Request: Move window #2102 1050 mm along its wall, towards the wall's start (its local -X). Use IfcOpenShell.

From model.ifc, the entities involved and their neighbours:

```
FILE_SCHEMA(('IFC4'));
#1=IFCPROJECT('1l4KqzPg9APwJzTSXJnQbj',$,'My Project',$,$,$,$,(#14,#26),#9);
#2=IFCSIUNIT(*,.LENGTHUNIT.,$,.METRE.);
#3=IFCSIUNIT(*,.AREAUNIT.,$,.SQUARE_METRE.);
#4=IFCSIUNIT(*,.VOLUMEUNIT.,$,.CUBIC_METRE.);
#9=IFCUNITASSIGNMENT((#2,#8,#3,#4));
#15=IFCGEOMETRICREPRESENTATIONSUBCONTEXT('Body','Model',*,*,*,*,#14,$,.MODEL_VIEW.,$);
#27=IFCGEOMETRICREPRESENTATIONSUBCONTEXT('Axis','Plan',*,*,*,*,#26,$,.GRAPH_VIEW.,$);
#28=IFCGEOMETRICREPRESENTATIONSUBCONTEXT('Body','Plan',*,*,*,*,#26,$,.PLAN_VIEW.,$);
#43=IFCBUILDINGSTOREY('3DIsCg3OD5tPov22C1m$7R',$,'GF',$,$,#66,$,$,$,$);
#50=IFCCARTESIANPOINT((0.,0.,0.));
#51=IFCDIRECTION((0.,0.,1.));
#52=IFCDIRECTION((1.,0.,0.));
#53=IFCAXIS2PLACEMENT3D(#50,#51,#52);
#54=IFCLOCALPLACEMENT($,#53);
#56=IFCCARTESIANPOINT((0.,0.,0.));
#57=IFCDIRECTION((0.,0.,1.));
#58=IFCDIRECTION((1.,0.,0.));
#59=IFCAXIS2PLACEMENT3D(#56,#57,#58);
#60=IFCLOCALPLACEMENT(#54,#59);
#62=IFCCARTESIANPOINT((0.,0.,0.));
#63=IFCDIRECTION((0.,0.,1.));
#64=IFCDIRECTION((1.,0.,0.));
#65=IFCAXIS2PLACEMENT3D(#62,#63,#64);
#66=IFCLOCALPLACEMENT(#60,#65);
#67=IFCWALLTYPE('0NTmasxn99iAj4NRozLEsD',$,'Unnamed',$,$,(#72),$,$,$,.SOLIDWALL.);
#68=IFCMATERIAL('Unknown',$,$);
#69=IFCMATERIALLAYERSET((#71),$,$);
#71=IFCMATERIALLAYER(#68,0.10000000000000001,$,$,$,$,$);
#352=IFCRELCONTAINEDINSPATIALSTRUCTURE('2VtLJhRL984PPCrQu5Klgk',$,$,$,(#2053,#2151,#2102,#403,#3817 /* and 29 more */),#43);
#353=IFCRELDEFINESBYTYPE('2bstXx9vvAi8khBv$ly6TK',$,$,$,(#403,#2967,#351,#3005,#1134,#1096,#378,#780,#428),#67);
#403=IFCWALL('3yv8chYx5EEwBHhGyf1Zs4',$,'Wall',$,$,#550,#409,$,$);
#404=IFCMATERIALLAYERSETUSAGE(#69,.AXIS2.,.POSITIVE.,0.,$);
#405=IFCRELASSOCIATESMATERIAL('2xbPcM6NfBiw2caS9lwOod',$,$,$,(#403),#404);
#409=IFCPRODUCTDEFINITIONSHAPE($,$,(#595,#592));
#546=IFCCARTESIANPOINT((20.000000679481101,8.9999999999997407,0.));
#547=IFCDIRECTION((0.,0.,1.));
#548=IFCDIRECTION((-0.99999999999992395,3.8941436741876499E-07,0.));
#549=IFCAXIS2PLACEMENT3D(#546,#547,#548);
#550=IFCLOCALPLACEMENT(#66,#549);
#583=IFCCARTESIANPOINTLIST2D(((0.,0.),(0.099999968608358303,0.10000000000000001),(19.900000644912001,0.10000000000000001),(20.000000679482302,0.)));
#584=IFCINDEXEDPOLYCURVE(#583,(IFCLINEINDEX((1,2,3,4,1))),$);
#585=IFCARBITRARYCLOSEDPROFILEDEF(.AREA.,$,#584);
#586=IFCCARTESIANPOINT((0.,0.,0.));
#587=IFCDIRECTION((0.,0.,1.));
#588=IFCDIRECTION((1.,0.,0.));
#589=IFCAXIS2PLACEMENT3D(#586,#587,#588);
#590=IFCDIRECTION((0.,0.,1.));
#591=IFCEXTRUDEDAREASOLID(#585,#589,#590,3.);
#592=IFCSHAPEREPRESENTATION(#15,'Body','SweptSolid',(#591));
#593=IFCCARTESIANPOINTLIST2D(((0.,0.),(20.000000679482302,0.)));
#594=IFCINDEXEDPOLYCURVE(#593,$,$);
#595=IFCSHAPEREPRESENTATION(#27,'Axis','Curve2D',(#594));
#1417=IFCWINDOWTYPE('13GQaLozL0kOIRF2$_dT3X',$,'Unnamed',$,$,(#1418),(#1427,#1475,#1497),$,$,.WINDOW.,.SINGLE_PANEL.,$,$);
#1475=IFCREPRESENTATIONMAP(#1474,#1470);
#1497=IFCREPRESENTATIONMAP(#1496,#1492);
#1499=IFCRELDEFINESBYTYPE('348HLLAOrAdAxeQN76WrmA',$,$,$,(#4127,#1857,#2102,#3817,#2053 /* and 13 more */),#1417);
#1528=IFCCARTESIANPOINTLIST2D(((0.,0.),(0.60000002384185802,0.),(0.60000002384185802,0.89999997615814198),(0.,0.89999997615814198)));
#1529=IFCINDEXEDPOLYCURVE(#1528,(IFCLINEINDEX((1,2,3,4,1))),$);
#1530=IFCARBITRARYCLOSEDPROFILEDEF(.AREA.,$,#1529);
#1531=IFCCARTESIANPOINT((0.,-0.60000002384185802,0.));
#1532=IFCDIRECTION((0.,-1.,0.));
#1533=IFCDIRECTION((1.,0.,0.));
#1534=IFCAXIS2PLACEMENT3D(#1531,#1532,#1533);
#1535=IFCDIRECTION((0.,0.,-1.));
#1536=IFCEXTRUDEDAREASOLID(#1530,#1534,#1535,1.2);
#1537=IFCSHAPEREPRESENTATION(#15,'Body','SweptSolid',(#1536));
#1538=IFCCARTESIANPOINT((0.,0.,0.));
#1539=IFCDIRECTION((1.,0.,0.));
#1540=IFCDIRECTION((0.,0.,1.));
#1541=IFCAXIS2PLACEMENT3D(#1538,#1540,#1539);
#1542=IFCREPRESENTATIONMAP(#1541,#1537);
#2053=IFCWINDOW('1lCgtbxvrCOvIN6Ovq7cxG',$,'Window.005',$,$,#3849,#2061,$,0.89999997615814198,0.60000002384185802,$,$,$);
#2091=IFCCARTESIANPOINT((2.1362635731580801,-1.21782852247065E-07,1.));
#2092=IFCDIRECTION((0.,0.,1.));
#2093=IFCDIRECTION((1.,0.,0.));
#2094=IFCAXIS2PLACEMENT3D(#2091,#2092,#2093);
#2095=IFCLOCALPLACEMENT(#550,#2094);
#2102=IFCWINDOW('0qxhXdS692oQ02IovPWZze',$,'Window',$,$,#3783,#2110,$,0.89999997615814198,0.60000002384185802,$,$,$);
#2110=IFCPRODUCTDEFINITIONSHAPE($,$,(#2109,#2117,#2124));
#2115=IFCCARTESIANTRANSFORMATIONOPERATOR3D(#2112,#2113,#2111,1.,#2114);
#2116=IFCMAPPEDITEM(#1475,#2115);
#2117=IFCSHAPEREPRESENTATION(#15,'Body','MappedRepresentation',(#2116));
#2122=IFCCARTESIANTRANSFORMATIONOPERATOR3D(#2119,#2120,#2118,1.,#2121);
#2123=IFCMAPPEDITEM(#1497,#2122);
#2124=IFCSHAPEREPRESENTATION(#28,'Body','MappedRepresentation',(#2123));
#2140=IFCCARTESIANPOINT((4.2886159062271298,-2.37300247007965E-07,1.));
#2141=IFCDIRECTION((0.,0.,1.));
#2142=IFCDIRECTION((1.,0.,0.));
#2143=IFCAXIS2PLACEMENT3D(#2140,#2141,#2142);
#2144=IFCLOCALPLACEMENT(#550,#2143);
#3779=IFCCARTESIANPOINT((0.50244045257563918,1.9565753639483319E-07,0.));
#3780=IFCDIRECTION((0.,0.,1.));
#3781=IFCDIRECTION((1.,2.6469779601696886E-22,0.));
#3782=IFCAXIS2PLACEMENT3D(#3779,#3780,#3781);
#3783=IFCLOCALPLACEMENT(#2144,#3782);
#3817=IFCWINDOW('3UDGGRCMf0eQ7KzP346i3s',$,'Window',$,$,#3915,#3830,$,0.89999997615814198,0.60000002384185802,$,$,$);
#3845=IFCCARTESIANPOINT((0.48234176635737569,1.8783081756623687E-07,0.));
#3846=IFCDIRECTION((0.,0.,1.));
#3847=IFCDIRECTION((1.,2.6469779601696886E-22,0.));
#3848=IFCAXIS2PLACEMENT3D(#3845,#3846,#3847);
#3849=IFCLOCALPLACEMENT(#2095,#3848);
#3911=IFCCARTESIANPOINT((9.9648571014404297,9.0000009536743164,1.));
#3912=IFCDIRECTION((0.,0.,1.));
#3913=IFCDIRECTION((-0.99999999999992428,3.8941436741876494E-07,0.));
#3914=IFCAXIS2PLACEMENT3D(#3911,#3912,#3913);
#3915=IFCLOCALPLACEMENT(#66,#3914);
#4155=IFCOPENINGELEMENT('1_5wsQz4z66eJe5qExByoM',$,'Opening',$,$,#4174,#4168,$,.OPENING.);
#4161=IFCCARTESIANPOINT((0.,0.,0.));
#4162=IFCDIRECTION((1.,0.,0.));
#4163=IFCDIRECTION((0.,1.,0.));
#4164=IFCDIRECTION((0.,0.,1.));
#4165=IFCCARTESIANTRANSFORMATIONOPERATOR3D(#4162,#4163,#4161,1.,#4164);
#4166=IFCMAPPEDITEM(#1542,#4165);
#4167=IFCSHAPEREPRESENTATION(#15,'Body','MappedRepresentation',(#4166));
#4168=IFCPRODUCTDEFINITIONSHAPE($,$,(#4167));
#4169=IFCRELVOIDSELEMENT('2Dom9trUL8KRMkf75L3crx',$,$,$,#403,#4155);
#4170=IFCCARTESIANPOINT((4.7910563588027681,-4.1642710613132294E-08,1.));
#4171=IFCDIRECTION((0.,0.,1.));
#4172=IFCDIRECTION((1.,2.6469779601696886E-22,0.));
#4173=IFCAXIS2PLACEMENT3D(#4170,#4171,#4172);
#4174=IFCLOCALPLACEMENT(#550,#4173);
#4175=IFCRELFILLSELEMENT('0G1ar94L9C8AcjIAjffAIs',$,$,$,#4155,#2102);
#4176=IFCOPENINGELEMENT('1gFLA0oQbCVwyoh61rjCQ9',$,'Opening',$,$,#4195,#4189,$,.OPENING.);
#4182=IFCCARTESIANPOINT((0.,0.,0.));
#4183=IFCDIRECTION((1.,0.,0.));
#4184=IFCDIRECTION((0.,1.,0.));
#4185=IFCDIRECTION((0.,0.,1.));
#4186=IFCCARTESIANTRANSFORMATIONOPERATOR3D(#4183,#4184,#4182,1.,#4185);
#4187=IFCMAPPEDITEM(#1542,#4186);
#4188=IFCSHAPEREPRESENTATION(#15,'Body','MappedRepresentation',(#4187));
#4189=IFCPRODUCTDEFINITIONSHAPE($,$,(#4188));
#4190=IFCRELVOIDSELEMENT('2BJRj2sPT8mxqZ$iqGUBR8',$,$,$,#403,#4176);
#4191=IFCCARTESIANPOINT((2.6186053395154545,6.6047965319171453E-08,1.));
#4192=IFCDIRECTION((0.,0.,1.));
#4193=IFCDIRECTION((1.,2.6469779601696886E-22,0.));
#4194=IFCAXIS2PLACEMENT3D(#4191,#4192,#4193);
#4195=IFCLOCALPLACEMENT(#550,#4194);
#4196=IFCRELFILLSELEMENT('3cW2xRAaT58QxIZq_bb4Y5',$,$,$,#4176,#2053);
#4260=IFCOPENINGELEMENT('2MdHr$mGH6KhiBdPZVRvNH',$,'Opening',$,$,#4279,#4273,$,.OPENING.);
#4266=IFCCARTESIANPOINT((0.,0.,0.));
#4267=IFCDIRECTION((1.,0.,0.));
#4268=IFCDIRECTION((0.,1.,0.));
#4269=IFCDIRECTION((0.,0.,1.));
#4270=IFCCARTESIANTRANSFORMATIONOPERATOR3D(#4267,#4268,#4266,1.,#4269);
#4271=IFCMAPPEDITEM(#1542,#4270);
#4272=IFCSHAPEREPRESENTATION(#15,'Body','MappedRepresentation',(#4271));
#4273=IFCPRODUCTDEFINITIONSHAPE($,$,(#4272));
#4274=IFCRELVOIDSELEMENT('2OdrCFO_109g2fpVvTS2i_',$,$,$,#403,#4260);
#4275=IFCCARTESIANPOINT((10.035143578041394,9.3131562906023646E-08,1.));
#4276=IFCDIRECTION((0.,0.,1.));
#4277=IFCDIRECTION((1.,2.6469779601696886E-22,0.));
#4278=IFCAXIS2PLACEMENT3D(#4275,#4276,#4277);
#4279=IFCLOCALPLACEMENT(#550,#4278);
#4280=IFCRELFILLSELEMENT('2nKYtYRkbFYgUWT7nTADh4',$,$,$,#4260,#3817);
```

```python
import ifcopenshell
import ifcopenshell.api.geometry
import ifcopenshell.util.placement
import ifcopenshell.util.unit

model = ifcopenshell.open("model.ifc")
unit_scale = ifcopenshell.util.unit.calculate_unit_scale(model)

window = model.by_guid("0qxhXdS692oQ02IovPWZze")
opening = window.FillsVoids[0].RelatingOpeningElement
wall = opening.VoidsElements[0].RelatingBuildingElement

wall_matrix = ifcopenshell.util.placement.get_local_placement(wall.ObjectPlacement)
shift = wall_matrix[:3, 0] * -1.05 / unit_scale
before = ifcopenshell.util.placement.get_local_placement(window.ObjectPlacement)[:3, 3].copy()

# The window is not placed relative to its opening, so move both.
for product in (opening, window):
    matrix = ifcopenshell.util.placement.get_local_placement(product.ObjectPlacement)
    matrix[:3, 3] += shift
    ifcopenshell.api.geometry.edit_object_placement(model, product=product, matrix=matrix, is_si=False)

after = ifcopenshell.util.placement.get_local_placement(window.ObjectPlacement)[:3, 3]
print("window moved by", (after - before).round(3) + 0.0)

model.write("model_v2.ifc")
```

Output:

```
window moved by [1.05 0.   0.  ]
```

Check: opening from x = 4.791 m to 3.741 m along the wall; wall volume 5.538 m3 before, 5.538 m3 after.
